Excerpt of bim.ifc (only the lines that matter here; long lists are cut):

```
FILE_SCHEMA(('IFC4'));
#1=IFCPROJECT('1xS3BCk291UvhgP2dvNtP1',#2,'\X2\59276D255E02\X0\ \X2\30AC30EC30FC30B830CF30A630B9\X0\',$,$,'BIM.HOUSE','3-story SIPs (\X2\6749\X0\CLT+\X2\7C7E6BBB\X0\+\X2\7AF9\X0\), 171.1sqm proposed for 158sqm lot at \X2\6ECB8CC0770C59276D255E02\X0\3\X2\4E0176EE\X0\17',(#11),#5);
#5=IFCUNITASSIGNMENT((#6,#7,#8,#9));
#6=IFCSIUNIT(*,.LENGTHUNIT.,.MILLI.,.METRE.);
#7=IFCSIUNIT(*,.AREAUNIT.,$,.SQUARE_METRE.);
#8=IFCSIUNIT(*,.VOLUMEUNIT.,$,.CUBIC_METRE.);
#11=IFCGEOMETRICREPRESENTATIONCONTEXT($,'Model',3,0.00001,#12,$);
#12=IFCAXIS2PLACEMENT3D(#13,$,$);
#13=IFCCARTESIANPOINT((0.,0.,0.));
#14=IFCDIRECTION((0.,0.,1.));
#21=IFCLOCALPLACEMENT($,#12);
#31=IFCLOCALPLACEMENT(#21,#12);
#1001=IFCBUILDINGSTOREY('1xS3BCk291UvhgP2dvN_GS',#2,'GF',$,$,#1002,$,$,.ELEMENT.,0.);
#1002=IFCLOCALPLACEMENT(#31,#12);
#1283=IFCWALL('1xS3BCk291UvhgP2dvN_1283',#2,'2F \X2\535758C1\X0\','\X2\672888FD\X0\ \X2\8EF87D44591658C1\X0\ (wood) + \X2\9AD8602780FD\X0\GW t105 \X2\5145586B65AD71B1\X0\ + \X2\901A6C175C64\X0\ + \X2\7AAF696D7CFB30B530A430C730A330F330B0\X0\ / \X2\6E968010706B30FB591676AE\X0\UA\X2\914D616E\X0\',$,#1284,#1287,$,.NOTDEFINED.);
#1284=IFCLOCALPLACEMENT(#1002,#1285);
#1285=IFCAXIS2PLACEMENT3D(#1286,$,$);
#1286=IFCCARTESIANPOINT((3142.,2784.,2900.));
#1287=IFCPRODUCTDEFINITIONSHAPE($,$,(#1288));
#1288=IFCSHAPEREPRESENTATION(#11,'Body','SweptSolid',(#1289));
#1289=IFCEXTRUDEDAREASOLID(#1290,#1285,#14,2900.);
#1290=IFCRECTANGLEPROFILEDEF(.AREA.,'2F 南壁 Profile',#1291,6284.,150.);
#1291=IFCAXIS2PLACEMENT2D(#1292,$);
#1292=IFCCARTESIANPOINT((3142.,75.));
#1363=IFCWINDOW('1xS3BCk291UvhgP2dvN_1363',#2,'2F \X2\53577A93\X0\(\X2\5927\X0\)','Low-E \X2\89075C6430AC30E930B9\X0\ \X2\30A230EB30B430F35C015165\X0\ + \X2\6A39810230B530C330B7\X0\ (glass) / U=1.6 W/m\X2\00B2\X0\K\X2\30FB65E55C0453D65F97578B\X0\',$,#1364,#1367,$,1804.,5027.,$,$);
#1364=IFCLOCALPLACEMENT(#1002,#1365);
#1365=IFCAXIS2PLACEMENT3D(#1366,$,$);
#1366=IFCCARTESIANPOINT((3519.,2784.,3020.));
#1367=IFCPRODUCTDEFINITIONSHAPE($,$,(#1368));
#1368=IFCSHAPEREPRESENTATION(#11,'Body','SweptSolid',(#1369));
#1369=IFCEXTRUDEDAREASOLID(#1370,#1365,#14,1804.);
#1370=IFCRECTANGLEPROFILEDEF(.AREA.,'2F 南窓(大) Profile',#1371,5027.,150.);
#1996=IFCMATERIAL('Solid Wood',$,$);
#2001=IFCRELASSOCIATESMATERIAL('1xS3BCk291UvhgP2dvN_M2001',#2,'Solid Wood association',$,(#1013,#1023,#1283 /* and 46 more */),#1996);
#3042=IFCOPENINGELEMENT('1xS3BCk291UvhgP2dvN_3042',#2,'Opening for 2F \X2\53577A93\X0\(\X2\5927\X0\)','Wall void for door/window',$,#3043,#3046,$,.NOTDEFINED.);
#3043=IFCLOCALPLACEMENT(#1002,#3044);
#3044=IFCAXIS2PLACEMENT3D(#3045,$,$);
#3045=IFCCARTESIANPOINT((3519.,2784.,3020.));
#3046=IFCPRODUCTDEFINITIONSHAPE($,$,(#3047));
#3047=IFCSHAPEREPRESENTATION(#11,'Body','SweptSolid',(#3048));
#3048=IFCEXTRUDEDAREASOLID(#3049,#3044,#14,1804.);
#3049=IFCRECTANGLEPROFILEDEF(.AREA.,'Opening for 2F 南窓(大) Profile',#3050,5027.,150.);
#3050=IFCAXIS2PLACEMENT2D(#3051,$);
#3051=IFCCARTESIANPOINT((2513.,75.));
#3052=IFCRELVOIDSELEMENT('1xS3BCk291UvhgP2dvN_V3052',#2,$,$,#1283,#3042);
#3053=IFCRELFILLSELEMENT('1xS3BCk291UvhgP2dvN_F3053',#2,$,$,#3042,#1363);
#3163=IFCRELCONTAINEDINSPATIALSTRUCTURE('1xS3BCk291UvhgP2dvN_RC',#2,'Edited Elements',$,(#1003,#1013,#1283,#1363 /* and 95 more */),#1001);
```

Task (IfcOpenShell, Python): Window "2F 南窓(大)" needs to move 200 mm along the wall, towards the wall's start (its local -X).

```python
import ifcopenshell
import ifcopenshell.api.geometry
import ifcopenshell.util.placement
import ifcopenshell.util.unit

model = ifcopenshell.open("bim.ifc")
unit_scale = ifcopenshell.util.unit.calculate_unit_scale(model)

window = model.by_guid("1xS3BCk291UvhgP2dvN_1363")
opening = window.FillsVoids[0].RelatingOpeningElement
wall = opening.VoidsElements[0].RelatingBuildingElement

wall_matrix = ifcopenshell.util.placement.get_local_placement(wall.ObjectPlacement)
shift = wall_matrix[:3, 0] * -0.2 / unit_scale
before = ifcopenshell.util.placement.get_local_placement(window.ObjectPlacement)[:3, 3].copy()

# The window is not placed relative to its opening, so move both.
for product in (opening, window):
    matrix = ifcopenshell.util.placement.get_local_placement(product.ObjectPlacement)
    matrix[:3, 3] += shift
    ifcopenshell.api.geometry.edit_object_placement(model, product=product, matrix=matrix, is_si=False)

after = ifcopenshell.util.placement.get_local_placement(window.ObjectPlacement)[:3, 3]
print("window moved by", (after - before).round(3) + 0.0)

model.write("bim_v2.ifc")
```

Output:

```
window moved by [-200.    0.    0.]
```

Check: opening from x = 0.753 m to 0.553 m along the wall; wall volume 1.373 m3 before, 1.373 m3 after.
